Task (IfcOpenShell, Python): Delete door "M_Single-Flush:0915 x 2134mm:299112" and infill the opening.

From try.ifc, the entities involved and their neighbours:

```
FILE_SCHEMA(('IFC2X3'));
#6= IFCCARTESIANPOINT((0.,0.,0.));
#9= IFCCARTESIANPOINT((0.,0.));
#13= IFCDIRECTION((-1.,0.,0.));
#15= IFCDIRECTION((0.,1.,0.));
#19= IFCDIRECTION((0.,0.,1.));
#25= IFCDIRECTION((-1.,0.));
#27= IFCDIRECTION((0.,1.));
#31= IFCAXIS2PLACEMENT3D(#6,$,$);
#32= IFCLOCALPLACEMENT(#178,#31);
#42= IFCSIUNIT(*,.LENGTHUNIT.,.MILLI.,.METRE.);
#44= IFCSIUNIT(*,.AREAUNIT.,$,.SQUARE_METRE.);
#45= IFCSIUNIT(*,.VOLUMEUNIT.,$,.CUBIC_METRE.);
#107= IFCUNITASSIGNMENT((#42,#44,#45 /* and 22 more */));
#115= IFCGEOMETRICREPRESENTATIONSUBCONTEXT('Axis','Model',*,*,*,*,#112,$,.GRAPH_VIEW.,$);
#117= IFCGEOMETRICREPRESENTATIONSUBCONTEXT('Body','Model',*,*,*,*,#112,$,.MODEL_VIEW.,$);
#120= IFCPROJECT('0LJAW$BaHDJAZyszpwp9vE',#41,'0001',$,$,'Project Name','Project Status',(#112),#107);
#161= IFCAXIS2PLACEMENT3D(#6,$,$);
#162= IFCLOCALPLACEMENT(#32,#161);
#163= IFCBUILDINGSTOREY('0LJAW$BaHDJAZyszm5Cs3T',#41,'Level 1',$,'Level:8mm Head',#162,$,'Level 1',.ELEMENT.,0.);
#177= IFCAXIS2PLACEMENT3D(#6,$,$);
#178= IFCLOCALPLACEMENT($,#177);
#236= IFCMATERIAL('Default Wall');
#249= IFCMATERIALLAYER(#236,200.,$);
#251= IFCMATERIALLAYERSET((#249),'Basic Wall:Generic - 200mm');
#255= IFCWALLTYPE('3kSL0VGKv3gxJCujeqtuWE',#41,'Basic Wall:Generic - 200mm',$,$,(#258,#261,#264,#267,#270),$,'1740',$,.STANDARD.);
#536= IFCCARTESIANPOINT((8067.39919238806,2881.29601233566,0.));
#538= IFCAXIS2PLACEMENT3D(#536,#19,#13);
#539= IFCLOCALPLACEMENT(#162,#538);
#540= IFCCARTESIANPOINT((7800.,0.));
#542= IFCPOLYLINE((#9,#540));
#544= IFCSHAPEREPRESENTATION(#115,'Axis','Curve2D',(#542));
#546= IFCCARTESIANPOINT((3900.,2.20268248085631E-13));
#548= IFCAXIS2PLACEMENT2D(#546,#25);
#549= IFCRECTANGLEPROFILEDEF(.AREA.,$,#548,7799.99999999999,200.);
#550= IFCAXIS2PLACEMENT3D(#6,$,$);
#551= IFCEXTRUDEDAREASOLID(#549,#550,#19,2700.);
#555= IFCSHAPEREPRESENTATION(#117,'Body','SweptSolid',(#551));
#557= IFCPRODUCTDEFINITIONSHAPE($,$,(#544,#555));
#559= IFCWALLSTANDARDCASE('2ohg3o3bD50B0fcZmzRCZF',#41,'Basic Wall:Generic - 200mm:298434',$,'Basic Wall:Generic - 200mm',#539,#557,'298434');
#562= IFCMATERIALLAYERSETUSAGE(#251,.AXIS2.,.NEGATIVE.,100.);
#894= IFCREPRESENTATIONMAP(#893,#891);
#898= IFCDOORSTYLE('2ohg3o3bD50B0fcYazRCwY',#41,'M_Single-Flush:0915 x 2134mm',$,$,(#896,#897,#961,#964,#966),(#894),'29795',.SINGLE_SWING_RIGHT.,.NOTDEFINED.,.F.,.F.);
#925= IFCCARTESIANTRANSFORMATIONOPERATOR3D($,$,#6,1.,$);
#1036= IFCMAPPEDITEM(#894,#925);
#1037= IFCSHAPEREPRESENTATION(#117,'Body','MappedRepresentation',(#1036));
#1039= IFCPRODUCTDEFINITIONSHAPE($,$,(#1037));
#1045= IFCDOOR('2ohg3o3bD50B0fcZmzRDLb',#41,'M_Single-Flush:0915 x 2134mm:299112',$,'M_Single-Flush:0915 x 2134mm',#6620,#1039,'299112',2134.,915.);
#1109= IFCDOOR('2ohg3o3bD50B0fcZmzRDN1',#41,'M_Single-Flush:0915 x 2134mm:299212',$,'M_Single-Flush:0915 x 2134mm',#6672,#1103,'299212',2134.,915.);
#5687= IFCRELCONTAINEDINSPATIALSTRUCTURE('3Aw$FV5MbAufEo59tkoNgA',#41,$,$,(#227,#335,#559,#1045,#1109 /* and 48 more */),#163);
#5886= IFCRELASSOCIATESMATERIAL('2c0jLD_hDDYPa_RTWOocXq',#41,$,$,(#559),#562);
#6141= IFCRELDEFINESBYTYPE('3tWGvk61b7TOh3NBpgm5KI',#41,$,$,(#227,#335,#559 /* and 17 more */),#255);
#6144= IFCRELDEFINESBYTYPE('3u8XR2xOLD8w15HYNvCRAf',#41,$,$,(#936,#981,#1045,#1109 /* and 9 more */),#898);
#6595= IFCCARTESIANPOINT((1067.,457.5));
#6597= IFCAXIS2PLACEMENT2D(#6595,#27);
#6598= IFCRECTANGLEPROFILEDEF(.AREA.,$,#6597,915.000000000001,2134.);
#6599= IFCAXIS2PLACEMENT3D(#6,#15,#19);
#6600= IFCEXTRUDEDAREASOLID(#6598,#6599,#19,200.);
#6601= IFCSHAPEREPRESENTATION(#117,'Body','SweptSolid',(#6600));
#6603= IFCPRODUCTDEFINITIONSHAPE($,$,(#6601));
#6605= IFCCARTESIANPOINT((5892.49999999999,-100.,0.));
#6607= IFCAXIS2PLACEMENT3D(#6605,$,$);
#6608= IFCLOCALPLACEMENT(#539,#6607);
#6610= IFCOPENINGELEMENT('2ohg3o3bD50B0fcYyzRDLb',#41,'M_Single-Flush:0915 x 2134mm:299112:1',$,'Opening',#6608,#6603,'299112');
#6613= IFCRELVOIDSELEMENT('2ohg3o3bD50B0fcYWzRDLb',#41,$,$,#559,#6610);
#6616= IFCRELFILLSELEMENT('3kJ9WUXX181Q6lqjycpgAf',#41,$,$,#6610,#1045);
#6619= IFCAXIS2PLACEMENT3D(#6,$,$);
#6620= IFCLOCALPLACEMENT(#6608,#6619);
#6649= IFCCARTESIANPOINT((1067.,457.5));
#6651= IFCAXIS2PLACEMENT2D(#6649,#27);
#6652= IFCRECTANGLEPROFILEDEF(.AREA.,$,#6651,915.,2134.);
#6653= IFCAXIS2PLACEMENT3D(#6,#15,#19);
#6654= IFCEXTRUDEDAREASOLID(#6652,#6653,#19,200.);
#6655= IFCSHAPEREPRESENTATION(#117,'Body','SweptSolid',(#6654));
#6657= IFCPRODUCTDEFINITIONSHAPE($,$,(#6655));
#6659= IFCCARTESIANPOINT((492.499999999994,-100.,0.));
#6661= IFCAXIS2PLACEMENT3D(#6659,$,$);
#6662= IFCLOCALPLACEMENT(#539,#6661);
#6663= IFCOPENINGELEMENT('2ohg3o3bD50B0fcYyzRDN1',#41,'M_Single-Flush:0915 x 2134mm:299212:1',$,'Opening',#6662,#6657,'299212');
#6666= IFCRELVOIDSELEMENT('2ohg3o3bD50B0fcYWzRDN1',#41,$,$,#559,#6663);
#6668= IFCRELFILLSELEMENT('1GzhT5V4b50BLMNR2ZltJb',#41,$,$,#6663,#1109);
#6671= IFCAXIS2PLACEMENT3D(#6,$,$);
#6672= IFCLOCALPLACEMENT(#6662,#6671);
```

```python
import ifcopenshell
import ifcopenshell.api.feature
import ifcopenshell.api.root
import ifcopenshell.geom
import ifcopenshell.util.shape

model = ifcopenshell.open("try.ifc")
settings = ifcopenshell.geom.settings()


def volume(element):
    """Net volume in cubic metres, openings subtracted."""
    shape = ifcopenshell.geom.create_shape(settings, element)
    return ifcopenshell.util.shape.get_volume(shape.geometry)


door = model.by_id(1045)
opening = door.FillsVoids[0].RelatingOpeningElement
wall = opening.VoidsElements[0].RelatingBuildingElement
before = volume(wall)

ifcopenshell.api.root.remove_product(model, product=door)
ifcopenshell.api.feature.remove_feature(model, feature=opening)

after = volume(wall)

print(f"wall volume {before:.3f} -> {after:.3f} m3")

model.write("try_edited.ifc")
```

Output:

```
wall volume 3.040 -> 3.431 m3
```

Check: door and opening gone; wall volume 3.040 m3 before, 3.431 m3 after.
